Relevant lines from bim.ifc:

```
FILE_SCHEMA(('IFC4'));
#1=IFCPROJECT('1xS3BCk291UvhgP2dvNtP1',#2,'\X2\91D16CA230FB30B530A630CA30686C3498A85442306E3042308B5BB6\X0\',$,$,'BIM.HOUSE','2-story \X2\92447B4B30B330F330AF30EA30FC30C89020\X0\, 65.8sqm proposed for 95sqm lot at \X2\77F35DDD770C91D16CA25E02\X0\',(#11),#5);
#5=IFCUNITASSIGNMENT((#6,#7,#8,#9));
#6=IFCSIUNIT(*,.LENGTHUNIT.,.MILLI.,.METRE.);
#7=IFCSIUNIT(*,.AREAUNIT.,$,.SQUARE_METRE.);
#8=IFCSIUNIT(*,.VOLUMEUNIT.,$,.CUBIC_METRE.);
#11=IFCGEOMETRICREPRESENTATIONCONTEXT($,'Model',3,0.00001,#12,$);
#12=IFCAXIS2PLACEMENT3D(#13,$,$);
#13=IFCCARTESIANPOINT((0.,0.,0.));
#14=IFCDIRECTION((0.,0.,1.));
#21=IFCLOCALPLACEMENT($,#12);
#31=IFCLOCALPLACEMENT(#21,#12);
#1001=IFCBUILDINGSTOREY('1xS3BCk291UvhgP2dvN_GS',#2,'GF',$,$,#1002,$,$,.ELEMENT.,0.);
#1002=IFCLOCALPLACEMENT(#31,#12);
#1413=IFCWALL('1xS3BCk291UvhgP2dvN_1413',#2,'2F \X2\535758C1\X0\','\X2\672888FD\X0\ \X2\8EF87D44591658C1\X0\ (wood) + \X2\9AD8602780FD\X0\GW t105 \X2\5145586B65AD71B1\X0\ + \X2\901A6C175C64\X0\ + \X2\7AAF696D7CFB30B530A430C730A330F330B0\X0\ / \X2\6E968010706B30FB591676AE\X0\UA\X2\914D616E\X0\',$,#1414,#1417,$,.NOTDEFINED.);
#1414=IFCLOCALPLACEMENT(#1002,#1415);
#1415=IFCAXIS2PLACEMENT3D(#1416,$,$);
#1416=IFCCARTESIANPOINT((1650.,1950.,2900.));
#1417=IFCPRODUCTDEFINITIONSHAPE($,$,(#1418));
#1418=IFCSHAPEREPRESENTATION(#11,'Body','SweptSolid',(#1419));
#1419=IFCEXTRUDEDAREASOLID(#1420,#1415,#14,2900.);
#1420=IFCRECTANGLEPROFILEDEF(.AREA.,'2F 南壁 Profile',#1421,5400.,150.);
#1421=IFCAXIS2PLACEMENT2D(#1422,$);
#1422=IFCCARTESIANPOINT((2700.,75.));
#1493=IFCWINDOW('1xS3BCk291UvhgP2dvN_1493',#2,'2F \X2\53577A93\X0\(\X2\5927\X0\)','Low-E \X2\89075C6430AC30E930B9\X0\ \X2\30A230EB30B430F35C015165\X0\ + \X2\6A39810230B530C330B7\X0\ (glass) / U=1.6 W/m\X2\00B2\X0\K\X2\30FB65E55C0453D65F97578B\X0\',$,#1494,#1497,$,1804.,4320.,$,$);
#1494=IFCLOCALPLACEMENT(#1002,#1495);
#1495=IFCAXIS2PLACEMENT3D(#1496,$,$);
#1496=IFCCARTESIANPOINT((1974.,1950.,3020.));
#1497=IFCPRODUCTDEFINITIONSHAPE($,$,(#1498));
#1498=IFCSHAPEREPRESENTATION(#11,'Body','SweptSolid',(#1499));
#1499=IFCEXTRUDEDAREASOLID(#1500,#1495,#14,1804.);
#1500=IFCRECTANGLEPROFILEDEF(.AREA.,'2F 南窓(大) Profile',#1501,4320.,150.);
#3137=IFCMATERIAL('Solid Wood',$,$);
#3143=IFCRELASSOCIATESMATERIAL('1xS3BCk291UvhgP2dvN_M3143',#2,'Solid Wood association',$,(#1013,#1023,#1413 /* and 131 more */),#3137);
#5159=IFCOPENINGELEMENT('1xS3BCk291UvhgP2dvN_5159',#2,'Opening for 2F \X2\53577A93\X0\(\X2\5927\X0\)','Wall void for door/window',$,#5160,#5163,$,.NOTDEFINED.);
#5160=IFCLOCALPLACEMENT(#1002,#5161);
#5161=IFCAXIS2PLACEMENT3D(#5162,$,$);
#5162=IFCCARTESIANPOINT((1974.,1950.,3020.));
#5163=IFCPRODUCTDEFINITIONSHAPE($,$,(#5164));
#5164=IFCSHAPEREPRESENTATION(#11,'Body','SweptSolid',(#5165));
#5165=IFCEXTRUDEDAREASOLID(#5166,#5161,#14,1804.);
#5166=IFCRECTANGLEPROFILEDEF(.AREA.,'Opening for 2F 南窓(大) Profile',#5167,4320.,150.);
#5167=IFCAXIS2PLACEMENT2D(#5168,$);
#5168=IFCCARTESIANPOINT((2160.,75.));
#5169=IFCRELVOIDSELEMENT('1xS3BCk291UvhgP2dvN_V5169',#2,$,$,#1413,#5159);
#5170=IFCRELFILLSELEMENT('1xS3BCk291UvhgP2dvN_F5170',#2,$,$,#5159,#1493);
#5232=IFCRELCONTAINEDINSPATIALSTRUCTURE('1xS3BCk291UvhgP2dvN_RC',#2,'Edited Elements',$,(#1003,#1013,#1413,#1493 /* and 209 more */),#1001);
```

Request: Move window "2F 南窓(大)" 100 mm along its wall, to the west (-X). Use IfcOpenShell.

```python
import ifcopenshell
import ifcopenshell.api.geometry
import ifcopenshell.util.placement
import ifcopenshell.util.unit

model = ifcopenshell.open("bim.ifc")
unit_scale = ifcopenshell.util.unit.calculate_unit_scale(model)

window = model.by_guid("1xS3BCk291UvhgP2dvN_1493")
opening = window.FillsVoids[0].RelatingOpeningElement
wall = opening.VoidsElements[0].RelatingBuildingElement

wall_matrix = ifcopenshell.util.placement.get_local_placement(wall.ObjectPlacement)
shift = wall_matrix[:3, 0] * -0.1 / unit_scale
before = ifcopenshell.util.placement.get_local_placement(window.ObjectPlacement)[:3, 3].copy()

# The window is not placed relative to its opening, so move both.
for product in (opening, window):
    matrix = ifcopenshell.util.placement.get_local_placement(product.ObjectPlacement)
    matrix[:3, 3] += shift
    ifcopenshell.api.geometry.edit_object_placement(model, product=product, matrix=matrix, is_si=False)

after = ifcopenshell.util.placement.get_local_placement(window.ObjectPlacement)[:3, 3]
print("window moved by", (after - before).round(3) + 0.0)

model.write("bim_updated.ifc")
```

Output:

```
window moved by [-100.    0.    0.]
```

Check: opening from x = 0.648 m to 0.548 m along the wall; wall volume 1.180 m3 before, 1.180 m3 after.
